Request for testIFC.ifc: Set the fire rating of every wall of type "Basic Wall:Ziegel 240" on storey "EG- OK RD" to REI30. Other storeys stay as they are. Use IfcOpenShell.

First a look at what the model holds.

```python
import ifcopenshell
import ifcopenshell.util.element

model = ifcopenshell.open("testIFC.ifc")
print(model.schema)
storey = next(s for s in model.by_type("IfcBuildingStorey") if s.Name == "EG- OK RD")
walls = [e for e in ifcopenshell.util.element.get_decomposition(storey) if e.is_a("IfcWall")]
seen = {}
for e in walls:
    element_type = ifcopenshell.util.element.get_type(e)
    key = (element_type.Name if element_type != e and element_type else None, ifcopenshell.util.element.get_pset(e, "Pset_WallCommon", "FireRating"))
    seen[key] = seen.get(key, 0) + 1
for (name, value), count in sorted(seen.items(), key=str):
    print(count, "x", name, "|", value)
```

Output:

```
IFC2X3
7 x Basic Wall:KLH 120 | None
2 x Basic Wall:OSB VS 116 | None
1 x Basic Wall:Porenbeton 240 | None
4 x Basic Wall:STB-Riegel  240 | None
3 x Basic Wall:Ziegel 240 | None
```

```python
import ifcopenshell
import ifcopenshell.api.pset
import ifcopenshell.util.element

model = ifcopenshell.open("testIFC.ifc")

storey = next(s for s in model.by_type("IfcBuildingStorey") if s.Name == "EG- OK RD")
walls = [e for e in ifcopenshell.util.element.get_decomposition(storey) if e.is_a("IfcWall")]

count = 0
for e in walls:
    element_type = ifcopenshell.util.element.get_type(e)
    if element_type in (None, e) or element_type.Name != "Basic Wall:Ziegel 240":
        continue
    # add_pset returns the element's existing set when there is one.
    pset = ifcopenshell.api.pset.add_pset(model, product=e, name="Pset_WallCommon")
    ifcopenshell.api.pset.edit_pset(model, pset=pset, properties={"FireRating": "REI30"})
    count += 1

print(count, "walls updated")

model.write("testIFC_edited.ifc")
```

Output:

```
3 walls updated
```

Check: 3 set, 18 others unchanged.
